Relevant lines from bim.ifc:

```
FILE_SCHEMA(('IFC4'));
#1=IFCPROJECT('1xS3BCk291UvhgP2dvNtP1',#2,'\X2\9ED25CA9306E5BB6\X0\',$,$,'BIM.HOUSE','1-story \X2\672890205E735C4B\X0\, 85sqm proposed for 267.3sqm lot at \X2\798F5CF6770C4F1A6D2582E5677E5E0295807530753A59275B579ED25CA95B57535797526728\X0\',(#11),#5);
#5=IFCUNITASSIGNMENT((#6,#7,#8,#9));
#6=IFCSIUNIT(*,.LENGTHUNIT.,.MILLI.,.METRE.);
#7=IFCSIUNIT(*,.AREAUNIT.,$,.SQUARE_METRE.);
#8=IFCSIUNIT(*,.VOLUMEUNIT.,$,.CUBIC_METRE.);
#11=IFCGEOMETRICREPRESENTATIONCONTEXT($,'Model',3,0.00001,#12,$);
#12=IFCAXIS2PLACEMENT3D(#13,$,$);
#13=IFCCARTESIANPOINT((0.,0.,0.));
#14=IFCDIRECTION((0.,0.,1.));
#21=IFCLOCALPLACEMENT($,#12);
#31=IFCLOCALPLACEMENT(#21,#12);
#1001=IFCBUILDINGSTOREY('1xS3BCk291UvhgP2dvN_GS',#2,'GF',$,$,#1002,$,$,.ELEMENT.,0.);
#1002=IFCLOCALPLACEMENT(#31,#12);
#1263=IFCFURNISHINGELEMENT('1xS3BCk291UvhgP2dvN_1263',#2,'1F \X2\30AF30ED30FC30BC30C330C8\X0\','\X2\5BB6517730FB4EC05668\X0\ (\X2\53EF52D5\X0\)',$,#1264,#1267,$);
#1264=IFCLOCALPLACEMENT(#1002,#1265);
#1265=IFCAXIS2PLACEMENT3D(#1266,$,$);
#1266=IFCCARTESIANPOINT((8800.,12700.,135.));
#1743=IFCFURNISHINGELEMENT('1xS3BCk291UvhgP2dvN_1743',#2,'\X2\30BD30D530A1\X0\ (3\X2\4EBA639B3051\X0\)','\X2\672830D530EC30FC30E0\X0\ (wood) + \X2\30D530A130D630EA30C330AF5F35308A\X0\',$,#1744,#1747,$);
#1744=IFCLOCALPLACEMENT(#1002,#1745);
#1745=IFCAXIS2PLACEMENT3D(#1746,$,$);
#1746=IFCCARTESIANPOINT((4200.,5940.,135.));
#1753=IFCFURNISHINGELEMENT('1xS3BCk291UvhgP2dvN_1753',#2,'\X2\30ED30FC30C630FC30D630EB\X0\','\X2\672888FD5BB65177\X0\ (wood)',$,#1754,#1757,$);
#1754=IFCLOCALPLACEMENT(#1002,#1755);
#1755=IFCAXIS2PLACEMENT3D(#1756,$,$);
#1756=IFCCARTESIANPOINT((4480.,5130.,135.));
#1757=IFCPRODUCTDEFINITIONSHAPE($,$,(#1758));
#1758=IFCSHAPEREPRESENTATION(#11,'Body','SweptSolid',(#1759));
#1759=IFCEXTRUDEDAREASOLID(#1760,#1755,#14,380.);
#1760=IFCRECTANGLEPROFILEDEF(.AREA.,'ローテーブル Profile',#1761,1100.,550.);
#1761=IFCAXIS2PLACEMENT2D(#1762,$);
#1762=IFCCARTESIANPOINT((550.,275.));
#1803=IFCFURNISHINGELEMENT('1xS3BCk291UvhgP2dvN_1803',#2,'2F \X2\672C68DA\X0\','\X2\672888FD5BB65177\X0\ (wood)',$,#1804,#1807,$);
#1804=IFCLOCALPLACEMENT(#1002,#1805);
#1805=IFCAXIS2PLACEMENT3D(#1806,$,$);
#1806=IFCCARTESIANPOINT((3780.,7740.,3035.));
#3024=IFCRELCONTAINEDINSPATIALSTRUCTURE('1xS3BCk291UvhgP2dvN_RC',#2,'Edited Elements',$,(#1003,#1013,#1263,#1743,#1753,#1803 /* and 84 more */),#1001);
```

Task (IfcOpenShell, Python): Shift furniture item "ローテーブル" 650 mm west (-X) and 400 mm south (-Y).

```python
import ifcopenshell
import ifcopenshell.api.geometry
import ifcopenshell.util.placement
import ifcopenshell.util.unit

model = ifcopenshell.open("bim.ifc")
unit_scale = ifcopenshell.util.unit.calculate_unit_scale(model)

item = model.by_guid("1xS3BCk291UvhgP2dvN_1753")
matrix = ifcopenshell.util.placement.get_local_placement(item.ObjectPlacement)
matrix[0, 3] -= 0.65 / unit_scale
matrix[1, 3] -= 0.4 / unit_scale
ifcopenshell.api.geometry.edit_object_placement(model, product=item, matrix=matrix, is_si=False)

print(ifcopenshell.util.placement.get_local_placement(item.ObjectPlacement).round(3) + 0.0)

model.write("bim_updated.ifc")
```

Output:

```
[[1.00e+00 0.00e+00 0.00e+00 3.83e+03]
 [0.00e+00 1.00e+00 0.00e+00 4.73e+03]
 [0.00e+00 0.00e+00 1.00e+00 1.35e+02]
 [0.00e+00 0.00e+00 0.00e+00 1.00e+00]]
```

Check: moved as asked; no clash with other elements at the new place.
